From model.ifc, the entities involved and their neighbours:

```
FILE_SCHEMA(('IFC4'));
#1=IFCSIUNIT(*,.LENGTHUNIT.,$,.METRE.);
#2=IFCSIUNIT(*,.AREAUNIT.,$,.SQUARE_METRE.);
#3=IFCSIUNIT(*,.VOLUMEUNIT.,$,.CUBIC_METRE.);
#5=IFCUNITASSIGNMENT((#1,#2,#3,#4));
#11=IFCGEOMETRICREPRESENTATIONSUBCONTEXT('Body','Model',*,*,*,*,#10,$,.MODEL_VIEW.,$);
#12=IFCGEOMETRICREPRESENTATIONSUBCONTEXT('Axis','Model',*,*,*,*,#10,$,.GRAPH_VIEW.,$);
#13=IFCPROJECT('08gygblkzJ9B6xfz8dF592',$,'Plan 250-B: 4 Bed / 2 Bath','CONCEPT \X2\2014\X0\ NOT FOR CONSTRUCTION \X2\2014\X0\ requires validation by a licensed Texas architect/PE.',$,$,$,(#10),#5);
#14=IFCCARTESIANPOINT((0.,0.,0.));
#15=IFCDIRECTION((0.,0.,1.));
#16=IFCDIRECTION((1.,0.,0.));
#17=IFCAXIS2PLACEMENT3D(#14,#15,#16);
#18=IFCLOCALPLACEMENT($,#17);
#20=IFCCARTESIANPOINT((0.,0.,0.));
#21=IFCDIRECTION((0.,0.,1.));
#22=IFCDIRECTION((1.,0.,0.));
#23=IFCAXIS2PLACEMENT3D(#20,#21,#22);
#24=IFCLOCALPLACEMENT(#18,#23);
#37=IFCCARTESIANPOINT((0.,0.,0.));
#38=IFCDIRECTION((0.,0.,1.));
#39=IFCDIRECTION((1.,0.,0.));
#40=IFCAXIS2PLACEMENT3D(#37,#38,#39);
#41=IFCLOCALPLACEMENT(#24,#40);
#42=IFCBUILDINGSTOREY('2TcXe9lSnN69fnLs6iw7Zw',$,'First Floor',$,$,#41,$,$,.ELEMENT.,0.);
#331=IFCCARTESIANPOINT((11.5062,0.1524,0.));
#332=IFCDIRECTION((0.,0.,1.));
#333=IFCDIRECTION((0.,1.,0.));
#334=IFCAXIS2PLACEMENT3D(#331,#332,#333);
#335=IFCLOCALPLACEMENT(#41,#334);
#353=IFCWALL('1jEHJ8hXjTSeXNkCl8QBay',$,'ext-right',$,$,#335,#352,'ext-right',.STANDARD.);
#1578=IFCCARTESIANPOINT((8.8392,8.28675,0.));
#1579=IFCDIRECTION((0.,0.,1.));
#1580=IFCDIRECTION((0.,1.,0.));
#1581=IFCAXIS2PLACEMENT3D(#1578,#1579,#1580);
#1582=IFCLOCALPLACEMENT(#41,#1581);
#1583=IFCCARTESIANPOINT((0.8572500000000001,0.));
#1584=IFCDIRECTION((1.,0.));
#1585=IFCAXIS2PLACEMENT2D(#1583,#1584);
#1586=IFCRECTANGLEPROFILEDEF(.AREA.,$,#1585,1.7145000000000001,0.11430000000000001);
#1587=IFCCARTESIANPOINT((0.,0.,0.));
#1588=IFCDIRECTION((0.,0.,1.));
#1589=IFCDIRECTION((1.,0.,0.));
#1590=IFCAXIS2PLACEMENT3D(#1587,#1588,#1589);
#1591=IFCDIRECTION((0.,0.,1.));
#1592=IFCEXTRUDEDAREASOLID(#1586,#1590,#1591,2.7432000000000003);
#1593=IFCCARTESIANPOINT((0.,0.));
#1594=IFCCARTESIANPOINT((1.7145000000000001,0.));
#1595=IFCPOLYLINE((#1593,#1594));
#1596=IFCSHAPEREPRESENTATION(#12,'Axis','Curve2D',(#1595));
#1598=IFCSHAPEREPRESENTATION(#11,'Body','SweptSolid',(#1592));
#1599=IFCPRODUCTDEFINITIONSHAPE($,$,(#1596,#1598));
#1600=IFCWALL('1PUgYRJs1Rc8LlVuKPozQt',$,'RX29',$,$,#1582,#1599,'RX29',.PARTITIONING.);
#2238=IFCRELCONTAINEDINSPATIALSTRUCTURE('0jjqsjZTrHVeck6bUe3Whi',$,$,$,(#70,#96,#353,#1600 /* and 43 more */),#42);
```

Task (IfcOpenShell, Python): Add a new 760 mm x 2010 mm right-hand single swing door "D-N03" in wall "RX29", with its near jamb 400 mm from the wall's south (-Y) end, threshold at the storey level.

```python
import numpy as np
import ifcopenshell
import ifcopenshell.api.feature
import ifcopenshell.api.geometry
import ifcopenshell.api.root
import ifcopenshell.api.spatial
import ifcopenshell.geom
import ifcopenshell.util.element
import ifcopenshell.util.placement
import ifcopenshell.util.representation
import ifcopenshell.util.shape
import ifcopenshell.util.unit

model = ifcopenshell.open("model.ifc")
unit_scale = ifcopenshell.util.unit.calculate_unit_scale(model)
settings = ifcopenshell.geom.settings()


def volume(element):
    """Net volume in cubic metres, openings subtracted."""
    shape = ifcopenshell.geom.create_shape(settings, element)
    return ifcopenshell.util.shape.get_volume(shape.geometry)


wall = model.by_guid("1PUgYRJs1Rc8LlVuKPozQt")
storey = ifcopenshell.util.element.get_container(wall, ifc_class="IfcBuildingStorey")
context = ifcopenshell.util.representation.get_context(model, "Model", "Body", "MODEL_VIEW")
before = volume(wall)

width, height, from_end, sill = 0.76, 2.01, 0.4, 0.0  # metres

# The wall runs along its own X axis, and the end named is its -X end.
wall_shape = ifcopenshell.geom.create_shape(settings, wall)
x, y, z = ifcopenshell.util.shape.get_vertices(wall_shape.geometry).T
start = x.min() + from_end
face, thickness = float(y.min()), float(y.max() - y.min())
wall_matrix = ifcopenshell.util.placement.get_local_placement(wall.ObjectPlacement)
level = ifcopenshell.util.placement.get_local_placement(storey.ObjectPlacement)[2, 3]


def in_wall(x, y):
    """Placement at x, y metres in the wall's axes, at sill height."""
    matrix = wall_matrix.copy()
    matrix[:, 3] = wall_matrix @ np.array([x / unit_scale, y / unit_scale, 0.0, 1.0])
    matrix[2, 3] = level + sill / unit_scale
    return matrix


# Opening: a box that overshoots both wall faces by 50 mm.
opening = ifcopenshell.api.root.create_entity(model, ifc_class="IfcOpeningElement", predefined_type="OPENING")
box = ifcopenshell.api.geometry.add_wall_representation(
    model, context=context, length=width, height=height, thickness=thickness + 0.1
)
ifcopenshell.api.geometry.assign_representation(model, product=opening, representation=box)
ifcopenshell.api.geometry.edit_object_placement(model, product=opening, matrix=in_wall(start, face - 0.05), is_si=False)
ifcopenshell.api.feature.add_feature(model, feature=opening, element=wall)

door = ifcopenshell.api.root.create_entity(model, ifc_class="IfcDoor", name="D-N03", predefined_type="DOOR")
door.OverallWidth, door.OverallHeight = width / unit_scale, height / unit_scale
door.OperationType = "SINGLE_SWING_RIGHT"
body = ifcopenshell.api.geometry.add_door_representation(
    model,
    context=context,
    overall_width=door.OverallWidth,
    overall_height=door.OverallHeight,
    operation_type="SINGLE_SWING_RIGHT",
    lining_properties={"LiningDepth": thickness / unit_scale, "ThresholdDepth": thickness / unit_scale},
)
ifcopenshell.api.geometry.assign_representation(model, product=door, representation=body)
ifcopenshell.api.spatial.assign_container(model, products=[door], relating_structure=storey)
ifcopenshell.api.feature.add_filling(model, opening=opening, element=door)

# The lining spans the wall, so the door starts at the wall face.
ifcopenshell.api.geometry.edit_object_placement(model, product=door, matrix=in_wall(start, face), is_si=False)

after = volume(wall)

print(f"wall volume {before:.3f} -> {after:.3f} m3")

model.write("model_v2.ifc")
```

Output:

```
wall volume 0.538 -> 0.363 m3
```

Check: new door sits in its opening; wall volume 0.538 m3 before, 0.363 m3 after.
